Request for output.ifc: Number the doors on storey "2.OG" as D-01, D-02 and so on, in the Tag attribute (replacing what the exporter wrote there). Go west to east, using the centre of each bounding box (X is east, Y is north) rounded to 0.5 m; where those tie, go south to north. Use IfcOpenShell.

First a look at what the model holds.

```python
import ifcopenshell
import ifcopenshell.util.element
import ifcopenshell.util.placement

model = ifcopenshell.open("output.ifc")
print(model.schema)
storey = next(s for s in model.by_type("IfcBuildingStorey") if s.Name == "2.OG")
doors = [e for e in ifcopenshell.util.element.get_decomposition(storey) if e.is_a("IfcDoor")]
for e in sorted(doors, key=lambda e: e.id()):
    origin = ifcopenshell.util.placement.get_local_placement(e.ObjectPlacement)[:3, 3]
    print(e.id(), e.Tag, e.Name, origin.round(2) + 0.0, sep=" | ")
```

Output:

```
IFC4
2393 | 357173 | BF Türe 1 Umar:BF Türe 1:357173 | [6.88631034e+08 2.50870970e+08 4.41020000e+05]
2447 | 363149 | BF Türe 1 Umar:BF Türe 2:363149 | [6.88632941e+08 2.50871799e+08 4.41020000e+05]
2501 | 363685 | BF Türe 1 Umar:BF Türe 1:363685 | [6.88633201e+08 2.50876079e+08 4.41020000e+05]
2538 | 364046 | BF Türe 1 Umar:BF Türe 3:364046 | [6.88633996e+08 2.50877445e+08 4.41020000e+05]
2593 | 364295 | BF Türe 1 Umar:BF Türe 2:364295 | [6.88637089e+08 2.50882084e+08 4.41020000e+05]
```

```python
import ifcopenshell
import ifcopenshell.geom
import ifcopenshell.util.element
import ifcopenshell.util.shape

model = ifcopenshell.open("output.ifc")
settings = ifcopenshell.geom.settings()
settings.set("use-world-coords", True)


def centre(element):
    shape = ifcopenshell.geom.create_shape(settings, element)
    return ifcopenshell.util.shape.get_bbox_centroid(shape.geometry)


storey = next(s for s in model.by_type("IfcBuildingStorey") if s.Name == "2.OG")
doors = [e for e in ifcopenshell.util.element.get_decomposition(storey) if e.is_a("IfcDoor")]

# Insertion points can sit at a corner or the storey origin, so sort by the geometry (in metres).
centres = {e: centre(e) for e in doors}
doors.sort(key=lambda e: (round(centres[e][0] / 0.5), centres[e][1]))

for i, e in enumerate(doors, start=1):
    number = f"D-{i:02d}"
    e.Tag = number
    print(e.id(), number)

model.write("output_updated.ifc")
```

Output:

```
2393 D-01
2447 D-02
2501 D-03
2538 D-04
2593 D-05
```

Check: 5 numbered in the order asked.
